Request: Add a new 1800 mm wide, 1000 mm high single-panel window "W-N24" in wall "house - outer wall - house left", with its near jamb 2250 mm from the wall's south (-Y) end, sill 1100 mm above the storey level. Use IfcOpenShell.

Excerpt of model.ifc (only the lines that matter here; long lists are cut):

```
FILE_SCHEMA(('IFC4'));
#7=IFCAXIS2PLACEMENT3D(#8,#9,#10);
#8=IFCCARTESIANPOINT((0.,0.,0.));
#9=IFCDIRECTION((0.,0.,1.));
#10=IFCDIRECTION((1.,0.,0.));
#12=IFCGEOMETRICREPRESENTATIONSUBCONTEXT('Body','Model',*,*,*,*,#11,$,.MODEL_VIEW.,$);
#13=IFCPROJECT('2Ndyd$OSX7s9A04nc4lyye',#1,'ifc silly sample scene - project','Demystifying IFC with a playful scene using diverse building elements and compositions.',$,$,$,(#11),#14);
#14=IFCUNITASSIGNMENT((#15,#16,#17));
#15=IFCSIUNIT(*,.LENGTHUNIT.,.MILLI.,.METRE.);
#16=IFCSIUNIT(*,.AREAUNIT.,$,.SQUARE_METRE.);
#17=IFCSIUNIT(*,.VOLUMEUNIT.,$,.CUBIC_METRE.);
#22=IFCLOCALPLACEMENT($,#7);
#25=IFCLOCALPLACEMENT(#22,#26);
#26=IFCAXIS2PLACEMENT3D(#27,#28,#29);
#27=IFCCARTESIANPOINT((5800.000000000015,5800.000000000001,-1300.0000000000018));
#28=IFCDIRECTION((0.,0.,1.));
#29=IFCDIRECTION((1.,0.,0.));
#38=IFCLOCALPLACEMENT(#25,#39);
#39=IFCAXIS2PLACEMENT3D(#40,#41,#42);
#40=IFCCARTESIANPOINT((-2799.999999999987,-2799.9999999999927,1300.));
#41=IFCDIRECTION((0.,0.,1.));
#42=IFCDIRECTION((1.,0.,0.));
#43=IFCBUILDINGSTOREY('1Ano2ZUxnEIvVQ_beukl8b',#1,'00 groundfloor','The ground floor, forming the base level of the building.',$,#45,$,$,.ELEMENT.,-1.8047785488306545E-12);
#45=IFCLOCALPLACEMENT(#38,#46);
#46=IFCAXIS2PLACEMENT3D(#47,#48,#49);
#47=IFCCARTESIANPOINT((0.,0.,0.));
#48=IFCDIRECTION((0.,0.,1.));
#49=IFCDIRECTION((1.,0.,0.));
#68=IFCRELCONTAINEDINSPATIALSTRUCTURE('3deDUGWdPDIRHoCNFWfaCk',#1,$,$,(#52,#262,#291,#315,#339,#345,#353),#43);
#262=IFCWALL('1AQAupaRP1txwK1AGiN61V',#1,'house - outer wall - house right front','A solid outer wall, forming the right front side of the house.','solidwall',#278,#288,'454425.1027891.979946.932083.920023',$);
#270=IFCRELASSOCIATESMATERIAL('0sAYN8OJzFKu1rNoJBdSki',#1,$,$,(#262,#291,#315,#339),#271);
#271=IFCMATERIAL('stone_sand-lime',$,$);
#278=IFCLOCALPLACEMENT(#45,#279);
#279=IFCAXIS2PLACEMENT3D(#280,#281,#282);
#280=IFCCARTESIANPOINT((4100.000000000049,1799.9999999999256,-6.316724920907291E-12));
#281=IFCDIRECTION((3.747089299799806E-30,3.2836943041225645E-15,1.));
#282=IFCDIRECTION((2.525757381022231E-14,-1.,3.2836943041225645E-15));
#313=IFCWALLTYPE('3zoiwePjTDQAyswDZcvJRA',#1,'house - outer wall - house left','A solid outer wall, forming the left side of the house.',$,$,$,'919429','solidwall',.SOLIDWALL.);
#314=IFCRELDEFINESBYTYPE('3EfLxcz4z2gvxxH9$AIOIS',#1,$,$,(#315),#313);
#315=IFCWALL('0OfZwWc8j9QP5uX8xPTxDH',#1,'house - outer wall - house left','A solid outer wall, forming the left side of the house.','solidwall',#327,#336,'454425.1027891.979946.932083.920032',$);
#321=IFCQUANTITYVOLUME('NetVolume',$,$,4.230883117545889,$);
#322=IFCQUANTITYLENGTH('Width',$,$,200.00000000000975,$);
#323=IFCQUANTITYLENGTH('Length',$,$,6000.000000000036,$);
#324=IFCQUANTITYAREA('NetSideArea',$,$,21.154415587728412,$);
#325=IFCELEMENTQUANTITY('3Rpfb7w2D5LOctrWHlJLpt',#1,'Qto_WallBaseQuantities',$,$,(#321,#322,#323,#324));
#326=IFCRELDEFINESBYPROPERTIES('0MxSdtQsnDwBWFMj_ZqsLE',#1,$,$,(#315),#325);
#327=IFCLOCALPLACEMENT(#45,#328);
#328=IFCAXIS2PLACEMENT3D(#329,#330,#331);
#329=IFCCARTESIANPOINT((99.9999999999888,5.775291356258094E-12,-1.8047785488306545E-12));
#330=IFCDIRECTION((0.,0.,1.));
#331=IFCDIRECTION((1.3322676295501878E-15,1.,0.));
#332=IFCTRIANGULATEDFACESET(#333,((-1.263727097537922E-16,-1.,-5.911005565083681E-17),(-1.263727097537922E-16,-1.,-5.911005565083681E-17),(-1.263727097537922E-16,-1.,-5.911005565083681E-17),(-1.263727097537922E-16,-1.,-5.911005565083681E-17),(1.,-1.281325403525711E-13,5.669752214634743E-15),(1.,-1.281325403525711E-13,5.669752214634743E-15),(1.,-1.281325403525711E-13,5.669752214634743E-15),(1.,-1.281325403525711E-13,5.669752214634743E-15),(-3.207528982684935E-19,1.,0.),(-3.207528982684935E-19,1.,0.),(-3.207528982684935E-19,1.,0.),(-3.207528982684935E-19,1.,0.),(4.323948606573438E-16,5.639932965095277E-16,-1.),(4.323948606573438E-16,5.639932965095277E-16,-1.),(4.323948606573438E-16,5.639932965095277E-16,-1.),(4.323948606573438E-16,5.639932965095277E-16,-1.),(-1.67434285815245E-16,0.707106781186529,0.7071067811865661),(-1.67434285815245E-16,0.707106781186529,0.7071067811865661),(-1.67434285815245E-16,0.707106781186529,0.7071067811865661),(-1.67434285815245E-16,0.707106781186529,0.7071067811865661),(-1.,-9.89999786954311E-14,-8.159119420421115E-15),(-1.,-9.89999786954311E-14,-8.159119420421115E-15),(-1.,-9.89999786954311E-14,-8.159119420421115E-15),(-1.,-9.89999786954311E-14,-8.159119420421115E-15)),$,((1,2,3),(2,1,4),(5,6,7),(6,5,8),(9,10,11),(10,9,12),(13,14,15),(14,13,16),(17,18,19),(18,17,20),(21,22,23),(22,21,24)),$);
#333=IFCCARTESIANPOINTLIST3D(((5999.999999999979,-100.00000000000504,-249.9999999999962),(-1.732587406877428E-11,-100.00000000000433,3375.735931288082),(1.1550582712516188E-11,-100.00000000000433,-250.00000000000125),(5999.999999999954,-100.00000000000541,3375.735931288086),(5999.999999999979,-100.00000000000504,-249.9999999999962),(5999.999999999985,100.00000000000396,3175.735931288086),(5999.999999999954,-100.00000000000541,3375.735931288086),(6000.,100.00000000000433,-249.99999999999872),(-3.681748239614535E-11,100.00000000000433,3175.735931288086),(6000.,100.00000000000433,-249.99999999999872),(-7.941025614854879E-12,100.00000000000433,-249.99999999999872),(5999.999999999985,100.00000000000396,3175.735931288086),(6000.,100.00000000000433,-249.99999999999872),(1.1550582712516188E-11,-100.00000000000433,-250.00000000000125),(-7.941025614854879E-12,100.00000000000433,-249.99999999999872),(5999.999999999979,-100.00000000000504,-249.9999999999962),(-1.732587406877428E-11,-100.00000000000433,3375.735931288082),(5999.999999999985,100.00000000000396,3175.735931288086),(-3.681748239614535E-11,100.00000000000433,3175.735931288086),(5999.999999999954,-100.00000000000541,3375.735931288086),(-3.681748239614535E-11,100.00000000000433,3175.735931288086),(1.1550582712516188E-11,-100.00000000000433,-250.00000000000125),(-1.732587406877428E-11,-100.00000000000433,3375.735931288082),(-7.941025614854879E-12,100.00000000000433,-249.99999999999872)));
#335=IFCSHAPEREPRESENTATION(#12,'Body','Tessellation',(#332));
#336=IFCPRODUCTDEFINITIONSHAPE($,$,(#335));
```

```python
import numpy as np
import ifcopenshell
import ifcopenshell.api.feature
import ifcopenshell.api.geometry
import ifcopenshell.api.pset
import ifcopenshell.api.root
import ifcopenshell.api.spatial
import ifcopenshell.geom
import ifcopenshell.util.element
import ifcopenshell.util.placement
import ifcopenshell.util.representation
import ifcopenshell.util.shape
import ifcopenshell.util.unit

model = ifcopenshell.open("model.ifc")
unit_scale = ifcopenshell.util.unit.calculate_unit_scale(model)
area_scale = ifcopenshell.util.unit.calculate_unit_scale(model, "AREAUNIT")
volume_scale = ifcopenshell.util.unit.calculate_unit_scale(model, "VOLUMEUNIT")
settings = ifcopenshell.geom.settings()


def volume(element):
    """Net volume in cubic metres, openings subtracted."""
    shape = ifcopenshell.geom.create_shape(settings, element)
    return ifcopenshell.util.shape.get_volume(shape.geometry)


wall = model.by_id(315)
storey = ifcopenshell.util.element.get_container(wall, ifc_class="IfcBuildingStorey")
context = ifcopenshell.util.representation.get_context(model, "Model", "Body", "MODEL_VIEW")
before = volume(wall)

width, height, from_end, sill = 1.8, 1, 2.25, 1.1  # metres

# The wall runs along its own X axis, and the end named is its -X end.
wall_shape = ifcopenshell.geom.create_shape(settings, wall)
x, y, z = ifcopenshell.util.shape.get_vertices(wall_shape.geometry).T
start = x.min() + from_end
face, thickness = float(y.min()), float(y.max() - y.min())
wall_matrix = ifcopenshell.util.placement.get_local_placement(wall.ObjectPlacement)
level = ifcopenshell.util.placement.get_local_placement(storey.ObjectPlacement)[2, 3]


def in_wall(x, y):
    """Placement at x, y metres in the wall's axes, at sill height."""
    matrix = wall_matrix.copy()
    matrix[:, 3] = wall_matrix @ np.array([x / unit_scale, y / unit_scale, 0.0, 1.0])
    matrix[2, 3] = level + sill / unit_scale
    return matrix


# Opening: a box that overshoots both wall faces by 50 mm.
opening = ifcopenshell.api.root.create_entity(model, ifc_class="IfcOpeningElement", predefined_type="OPENING")
box = ifcopenshell.api.geometry.add_wall_representation(
    model, context=context, length=width, height=height, thickness=thickness + 0.1
)
ifcopenshell.api.geometry.assign_representation(model, product=opening, representation=box)
ifcopenshell.api.geometry.edit_object_placement(model, product=opening, matrix=in_wall(start, face - 0.05), is_si=False)
ifcopenshell.api.feature.add_feature(model, feature=opening, element=wall)

window = ifcopenshell.api.root.create_entity(model, ifc_class="IfcWindow", name="W-N24", predefined_type="WINDOW")
window.OverallWidth, window.OverallHeight = width / unit_scale, height / unit_scale
window.PartitioningType = "SINGLE_PANEL"
body = ifcopenshell.api.geometry.add_window_representation(
    model,
    context=context,
    overall_width=window.OverallWidth,
    overall_height=window.OverallHeight,
    partition_type="SINGLE_PANEL",
)
ifcopenshell.api.geometry.assign_representation(model, product=window, representation=body)
ifcopenshell.api.spatial.assign_container(model, products=[window], relating_structure=storey)
ifcopenshell.api.feature.add_filling(model, opening=opening, element=window)

# Centre the window in the wall's thickness.
ifcopenshell.api.geometry.edit_object_placement(model, product=window, matrix=in_wall(start, face), is_si=False)
window_shape = ifcopenshell.geom.create_shape(settings, window)
depth = ifcopenshell.util.shape.get_vertices(window_shape.geometry)[:, 1]
offset = face + thickness / 2 - (depth.min() + depth.max()) / 2
ifcopenshell.api.geometry.edit_object_placement(model, product=window, matrix=in_wall(start, offset), is_si=False)

after = volume(wall)

# Update the wall's stored quantities.
qto = model.by_id(ifcopenshell.util.element.get_pset(wall, "Qto_WallBaseQuantities", should_inherit=False)["id"])
ifcopenshell.api.pset.edit_qto(model, qto=qto, properties={
    "NetVolume": after / volume_scale,
    "NetSideArea": after / thickness / area_scale,
})

print(f"wall volume {before:.3f} -> {after:.3f} m3")

model.write("model_rev.ifc")
```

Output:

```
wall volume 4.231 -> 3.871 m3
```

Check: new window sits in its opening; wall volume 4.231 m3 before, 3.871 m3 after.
